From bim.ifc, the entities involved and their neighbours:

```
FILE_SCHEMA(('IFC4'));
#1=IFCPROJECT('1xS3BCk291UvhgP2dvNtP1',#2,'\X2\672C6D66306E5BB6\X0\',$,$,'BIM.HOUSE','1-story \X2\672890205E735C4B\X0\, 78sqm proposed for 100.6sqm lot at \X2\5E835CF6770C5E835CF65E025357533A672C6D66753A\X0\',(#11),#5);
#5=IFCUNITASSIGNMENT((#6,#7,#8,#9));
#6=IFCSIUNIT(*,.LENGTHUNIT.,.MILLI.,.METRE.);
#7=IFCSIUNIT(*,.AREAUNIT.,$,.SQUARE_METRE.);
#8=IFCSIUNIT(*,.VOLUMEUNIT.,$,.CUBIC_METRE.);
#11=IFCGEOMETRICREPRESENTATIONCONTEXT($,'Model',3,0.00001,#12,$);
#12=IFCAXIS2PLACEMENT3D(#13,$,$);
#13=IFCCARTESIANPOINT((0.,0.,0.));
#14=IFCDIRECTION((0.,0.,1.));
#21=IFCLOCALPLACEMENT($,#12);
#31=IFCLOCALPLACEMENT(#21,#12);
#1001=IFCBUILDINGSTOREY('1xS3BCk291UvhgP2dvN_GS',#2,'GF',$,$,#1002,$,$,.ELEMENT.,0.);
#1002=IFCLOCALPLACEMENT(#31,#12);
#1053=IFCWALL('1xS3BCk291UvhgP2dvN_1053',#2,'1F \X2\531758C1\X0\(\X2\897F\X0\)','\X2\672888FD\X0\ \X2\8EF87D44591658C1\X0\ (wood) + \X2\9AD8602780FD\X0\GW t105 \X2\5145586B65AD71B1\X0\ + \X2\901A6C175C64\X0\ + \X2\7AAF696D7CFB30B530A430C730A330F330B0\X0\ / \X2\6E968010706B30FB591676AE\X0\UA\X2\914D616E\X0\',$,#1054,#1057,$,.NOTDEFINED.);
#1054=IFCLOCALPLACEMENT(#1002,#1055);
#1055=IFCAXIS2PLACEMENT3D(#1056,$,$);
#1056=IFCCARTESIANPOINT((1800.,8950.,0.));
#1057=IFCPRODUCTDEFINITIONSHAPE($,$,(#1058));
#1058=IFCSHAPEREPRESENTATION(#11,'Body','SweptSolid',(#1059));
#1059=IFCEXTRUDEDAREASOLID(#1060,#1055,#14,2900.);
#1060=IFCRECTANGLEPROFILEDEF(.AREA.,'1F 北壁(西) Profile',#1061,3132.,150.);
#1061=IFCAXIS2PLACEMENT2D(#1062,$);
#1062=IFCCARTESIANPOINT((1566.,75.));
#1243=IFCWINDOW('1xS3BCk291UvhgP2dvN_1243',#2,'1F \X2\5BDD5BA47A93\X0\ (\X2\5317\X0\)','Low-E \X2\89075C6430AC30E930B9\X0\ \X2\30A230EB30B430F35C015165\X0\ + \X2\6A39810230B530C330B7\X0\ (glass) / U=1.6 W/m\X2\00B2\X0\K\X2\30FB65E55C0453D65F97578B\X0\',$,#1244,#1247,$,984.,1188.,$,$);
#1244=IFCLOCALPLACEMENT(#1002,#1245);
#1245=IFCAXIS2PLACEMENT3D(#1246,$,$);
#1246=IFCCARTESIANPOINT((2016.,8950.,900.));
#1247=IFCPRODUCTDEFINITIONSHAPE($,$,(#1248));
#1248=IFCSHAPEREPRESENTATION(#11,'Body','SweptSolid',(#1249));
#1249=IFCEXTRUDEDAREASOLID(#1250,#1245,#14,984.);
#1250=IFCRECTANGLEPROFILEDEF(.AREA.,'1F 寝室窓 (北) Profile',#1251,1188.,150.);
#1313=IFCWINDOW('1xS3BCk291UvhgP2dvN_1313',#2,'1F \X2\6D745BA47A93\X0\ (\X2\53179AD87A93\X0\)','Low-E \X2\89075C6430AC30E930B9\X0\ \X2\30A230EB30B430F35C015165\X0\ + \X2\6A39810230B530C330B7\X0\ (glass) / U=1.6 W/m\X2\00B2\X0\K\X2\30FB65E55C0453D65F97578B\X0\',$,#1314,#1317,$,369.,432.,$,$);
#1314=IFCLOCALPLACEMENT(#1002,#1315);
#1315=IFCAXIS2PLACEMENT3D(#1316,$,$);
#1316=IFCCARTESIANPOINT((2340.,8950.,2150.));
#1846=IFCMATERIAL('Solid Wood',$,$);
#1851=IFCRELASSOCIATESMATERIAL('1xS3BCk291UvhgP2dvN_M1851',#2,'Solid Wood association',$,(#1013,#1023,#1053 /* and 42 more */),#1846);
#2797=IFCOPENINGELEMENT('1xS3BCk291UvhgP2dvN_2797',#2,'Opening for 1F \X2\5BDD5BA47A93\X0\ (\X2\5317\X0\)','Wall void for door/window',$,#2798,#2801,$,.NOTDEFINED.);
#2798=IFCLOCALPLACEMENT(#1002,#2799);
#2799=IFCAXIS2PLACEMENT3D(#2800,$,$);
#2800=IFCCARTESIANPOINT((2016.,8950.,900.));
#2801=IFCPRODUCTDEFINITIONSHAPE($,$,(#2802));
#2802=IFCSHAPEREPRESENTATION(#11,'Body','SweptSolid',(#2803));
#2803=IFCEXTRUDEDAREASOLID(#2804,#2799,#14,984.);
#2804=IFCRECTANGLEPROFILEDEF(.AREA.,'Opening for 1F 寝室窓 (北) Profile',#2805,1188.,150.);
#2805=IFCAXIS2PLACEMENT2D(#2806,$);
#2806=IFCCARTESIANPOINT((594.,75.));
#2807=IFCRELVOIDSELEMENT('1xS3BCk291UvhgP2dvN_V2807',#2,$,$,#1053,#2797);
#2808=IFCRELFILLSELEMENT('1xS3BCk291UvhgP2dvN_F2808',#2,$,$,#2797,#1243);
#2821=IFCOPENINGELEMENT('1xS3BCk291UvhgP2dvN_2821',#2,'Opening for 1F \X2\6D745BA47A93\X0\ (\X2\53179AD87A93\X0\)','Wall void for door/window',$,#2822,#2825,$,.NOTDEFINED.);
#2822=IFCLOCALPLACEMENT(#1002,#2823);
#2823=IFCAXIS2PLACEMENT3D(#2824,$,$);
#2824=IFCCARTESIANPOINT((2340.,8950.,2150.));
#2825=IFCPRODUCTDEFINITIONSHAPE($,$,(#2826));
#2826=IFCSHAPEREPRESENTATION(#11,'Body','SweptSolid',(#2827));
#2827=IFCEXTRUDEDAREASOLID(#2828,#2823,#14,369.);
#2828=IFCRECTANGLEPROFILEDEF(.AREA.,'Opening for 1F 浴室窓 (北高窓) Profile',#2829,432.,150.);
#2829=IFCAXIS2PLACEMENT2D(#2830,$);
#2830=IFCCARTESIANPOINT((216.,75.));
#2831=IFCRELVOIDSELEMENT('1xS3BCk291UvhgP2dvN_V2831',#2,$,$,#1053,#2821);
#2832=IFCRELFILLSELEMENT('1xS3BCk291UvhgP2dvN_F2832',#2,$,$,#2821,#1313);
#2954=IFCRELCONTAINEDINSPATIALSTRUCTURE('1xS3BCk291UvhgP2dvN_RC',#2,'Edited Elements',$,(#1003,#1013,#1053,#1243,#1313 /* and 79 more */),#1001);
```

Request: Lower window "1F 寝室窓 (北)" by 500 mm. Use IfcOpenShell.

```python
import numpy as np
import ifcopenshell
import ifcopenshell.api.geometry
import ifcopenshell.util.placement
import ifcopenshell.util.unit

model = ifcopenshell.open("bim.ifc")
unit_scale = ifcopenshell.util.unit.calculate_unit_scale(model)

window = model.by_guid("1xS3BCk291UvhgP2dvN_1243")
opening = window.FillsVoids[0].RelatingOpeningElement
dz = -500.0

shift = np.array([0.0, 0.0, dz])
# The window is not placed relative to its opening, so move both.
for product in (opening, window):
    matrix = ifcopenshell.util.placement.get_local_placement(product.ObjectPlacement)
    matrix[:3, 3] += shift
    ifcopenshell.api.geometry.edit_object_placement(model, product=product, matrix=matrix, is_si=False)

print(f"moved by {dz * unit_scale:+.3f} m")

model.write("bim_updated.ifc")
```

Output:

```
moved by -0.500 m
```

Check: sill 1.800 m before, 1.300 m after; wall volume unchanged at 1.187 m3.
